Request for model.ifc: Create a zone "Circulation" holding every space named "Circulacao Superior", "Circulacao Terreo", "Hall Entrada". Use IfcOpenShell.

First a look at what the model holds.

```python
import ifcopenshell

model = ifcopenshell.open("model.ifc")
print(model.schema)
seen = {}
for space in model.by_type("IfcSpace"):
    seen[space.Name] = seen.get(space.Name, 0) + 1
for name, count in sorted(seen.items(), key=str):
    print(count, "x", name)
print("zones:", [z.Name for z in model.by_type("IfcZone")][:20])
```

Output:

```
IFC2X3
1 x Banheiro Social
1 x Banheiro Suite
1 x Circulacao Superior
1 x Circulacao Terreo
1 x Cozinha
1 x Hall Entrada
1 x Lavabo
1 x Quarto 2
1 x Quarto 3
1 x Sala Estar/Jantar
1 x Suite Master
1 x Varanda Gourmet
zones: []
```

```python
import ifcopenshell
import ifcopenshell.api.group
import ifcopenshell.api.root

model = ifcopenshell.open("model.ifc")

names = {"Circulacao Superior", "Circulacao Terreo", "Hall Entrada"}
spaces = [s for s in model.by_type("IfcSpace") if s.Name in names]

zone = ifcopenshell.api.root.create_entity(model, ifc_class="IfcZone", name="Circulation")
ifcopenshell.api.group.assign_group(model, products=spaces, group=zone)
print(len(spaces), "spaces in", zone.Name)

model.write("model_v2.ifc")
```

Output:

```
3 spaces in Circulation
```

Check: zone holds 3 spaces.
